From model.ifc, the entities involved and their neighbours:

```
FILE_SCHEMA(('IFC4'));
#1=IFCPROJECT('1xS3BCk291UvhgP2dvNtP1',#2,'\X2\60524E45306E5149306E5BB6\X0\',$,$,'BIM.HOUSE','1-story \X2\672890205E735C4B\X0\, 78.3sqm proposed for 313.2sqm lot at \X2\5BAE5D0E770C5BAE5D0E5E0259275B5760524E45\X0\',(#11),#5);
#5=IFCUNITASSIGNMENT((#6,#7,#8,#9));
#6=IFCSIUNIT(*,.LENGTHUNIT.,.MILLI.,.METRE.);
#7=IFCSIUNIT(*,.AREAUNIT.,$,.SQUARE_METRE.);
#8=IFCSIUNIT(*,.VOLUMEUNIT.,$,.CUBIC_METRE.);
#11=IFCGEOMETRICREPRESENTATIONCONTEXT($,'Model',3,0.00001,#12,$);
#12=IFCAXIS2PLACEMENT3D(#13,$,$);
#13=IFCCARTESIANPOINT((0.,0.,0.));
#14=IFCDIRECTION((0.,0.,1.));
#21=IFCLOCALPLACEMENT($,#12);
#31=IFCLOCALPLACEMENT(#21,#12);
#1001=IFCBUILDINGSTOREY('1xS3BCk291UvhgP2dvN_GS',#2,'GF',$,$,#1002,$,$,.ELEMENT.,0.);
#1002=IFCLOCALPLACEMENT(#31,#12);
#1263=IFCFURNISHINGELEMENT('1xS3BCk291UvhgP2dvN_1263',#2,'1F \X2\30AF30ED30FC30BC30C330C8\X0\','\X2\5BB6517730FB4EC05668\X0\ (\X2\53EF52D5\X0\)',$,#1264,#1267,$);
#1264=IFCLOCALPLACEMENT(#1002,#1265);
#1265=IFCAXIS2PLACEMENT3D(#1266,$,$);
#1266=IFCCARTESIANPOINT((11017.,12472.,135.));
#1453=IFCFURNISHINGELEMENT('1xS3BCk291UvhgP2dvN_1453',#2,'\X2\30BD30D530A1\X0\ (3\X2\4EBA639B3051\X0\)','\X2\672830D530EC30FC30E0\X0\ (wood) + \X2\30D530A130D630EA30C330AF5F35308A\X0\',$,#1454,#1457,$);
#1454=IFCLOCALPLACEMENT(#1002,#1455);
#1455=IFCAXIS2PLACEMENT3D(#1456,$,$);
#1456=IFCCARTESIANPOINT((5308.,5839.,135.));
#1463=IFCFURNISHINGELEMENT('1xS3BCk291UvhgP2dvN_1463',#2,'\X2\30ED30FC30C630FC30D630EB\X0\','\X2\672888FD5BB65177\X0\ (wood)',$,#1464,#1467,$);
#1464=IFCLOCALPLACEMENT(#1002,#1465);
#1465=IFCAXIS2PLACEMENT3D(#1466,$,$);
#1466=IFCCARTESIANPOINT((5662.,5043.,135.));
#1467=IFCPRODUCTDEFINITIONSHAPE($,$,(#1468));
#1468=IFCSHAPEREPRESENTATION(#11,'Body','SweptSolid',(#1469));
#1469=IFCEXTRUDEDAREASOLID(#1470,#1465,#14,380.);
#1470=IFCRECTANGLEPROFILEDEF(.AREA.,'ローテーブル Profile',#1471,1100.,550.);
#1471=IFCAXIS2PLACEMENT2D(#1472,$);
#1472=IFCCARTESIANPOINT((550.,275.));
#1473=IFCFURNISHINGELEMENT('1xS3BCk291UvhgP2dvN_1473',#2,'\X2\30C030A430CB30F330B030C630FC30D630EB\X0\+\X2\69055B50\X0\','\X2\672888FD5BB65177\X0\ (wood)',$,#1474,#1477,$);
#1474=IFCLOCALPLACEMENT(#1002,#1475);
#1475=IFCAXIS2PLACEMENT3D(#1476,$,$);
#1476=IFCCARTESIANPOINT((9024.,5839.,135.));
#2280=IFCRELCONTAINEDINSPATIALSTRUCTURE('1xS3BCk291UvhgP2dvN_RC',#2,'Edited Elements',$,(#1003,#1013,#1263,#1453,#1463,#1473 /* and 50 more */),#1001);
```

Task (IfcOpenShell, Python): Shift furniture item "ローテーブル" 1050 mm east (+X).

```python
import ifcopenshell
import ifcopenshell.api.geometry
import ifcopenshell.util.placement
import ifcopenshell.util.unit

model = ifcopenshell.open("model.ifc")
unit_scale = ifcopenshell.util.unit.calculate_unit_scale(model)

item = model.by_id(1463)
matrix = ifcopenshell.util.placement.get_local_placement(item.ObjectPlacement)
matrix[0, 3] += 1.05 / unit_scale
ifcopenshell.api.geometry.edit_object_placement(model, product=item, matrix=matrix, is_si=False)

print(ifcopenshell.util.placement.get_local_placement(item.ObjectPlacement).round(3) + 0.0)

model.write("model_rev.ifc")
```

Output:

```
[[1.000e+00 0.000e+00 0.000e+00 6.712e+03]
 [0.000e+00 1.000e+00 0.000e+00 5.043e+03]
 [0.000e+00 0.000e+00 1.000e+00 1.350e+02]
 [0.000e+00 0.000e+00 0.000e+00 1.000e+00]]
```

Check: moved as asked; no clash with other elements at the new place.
